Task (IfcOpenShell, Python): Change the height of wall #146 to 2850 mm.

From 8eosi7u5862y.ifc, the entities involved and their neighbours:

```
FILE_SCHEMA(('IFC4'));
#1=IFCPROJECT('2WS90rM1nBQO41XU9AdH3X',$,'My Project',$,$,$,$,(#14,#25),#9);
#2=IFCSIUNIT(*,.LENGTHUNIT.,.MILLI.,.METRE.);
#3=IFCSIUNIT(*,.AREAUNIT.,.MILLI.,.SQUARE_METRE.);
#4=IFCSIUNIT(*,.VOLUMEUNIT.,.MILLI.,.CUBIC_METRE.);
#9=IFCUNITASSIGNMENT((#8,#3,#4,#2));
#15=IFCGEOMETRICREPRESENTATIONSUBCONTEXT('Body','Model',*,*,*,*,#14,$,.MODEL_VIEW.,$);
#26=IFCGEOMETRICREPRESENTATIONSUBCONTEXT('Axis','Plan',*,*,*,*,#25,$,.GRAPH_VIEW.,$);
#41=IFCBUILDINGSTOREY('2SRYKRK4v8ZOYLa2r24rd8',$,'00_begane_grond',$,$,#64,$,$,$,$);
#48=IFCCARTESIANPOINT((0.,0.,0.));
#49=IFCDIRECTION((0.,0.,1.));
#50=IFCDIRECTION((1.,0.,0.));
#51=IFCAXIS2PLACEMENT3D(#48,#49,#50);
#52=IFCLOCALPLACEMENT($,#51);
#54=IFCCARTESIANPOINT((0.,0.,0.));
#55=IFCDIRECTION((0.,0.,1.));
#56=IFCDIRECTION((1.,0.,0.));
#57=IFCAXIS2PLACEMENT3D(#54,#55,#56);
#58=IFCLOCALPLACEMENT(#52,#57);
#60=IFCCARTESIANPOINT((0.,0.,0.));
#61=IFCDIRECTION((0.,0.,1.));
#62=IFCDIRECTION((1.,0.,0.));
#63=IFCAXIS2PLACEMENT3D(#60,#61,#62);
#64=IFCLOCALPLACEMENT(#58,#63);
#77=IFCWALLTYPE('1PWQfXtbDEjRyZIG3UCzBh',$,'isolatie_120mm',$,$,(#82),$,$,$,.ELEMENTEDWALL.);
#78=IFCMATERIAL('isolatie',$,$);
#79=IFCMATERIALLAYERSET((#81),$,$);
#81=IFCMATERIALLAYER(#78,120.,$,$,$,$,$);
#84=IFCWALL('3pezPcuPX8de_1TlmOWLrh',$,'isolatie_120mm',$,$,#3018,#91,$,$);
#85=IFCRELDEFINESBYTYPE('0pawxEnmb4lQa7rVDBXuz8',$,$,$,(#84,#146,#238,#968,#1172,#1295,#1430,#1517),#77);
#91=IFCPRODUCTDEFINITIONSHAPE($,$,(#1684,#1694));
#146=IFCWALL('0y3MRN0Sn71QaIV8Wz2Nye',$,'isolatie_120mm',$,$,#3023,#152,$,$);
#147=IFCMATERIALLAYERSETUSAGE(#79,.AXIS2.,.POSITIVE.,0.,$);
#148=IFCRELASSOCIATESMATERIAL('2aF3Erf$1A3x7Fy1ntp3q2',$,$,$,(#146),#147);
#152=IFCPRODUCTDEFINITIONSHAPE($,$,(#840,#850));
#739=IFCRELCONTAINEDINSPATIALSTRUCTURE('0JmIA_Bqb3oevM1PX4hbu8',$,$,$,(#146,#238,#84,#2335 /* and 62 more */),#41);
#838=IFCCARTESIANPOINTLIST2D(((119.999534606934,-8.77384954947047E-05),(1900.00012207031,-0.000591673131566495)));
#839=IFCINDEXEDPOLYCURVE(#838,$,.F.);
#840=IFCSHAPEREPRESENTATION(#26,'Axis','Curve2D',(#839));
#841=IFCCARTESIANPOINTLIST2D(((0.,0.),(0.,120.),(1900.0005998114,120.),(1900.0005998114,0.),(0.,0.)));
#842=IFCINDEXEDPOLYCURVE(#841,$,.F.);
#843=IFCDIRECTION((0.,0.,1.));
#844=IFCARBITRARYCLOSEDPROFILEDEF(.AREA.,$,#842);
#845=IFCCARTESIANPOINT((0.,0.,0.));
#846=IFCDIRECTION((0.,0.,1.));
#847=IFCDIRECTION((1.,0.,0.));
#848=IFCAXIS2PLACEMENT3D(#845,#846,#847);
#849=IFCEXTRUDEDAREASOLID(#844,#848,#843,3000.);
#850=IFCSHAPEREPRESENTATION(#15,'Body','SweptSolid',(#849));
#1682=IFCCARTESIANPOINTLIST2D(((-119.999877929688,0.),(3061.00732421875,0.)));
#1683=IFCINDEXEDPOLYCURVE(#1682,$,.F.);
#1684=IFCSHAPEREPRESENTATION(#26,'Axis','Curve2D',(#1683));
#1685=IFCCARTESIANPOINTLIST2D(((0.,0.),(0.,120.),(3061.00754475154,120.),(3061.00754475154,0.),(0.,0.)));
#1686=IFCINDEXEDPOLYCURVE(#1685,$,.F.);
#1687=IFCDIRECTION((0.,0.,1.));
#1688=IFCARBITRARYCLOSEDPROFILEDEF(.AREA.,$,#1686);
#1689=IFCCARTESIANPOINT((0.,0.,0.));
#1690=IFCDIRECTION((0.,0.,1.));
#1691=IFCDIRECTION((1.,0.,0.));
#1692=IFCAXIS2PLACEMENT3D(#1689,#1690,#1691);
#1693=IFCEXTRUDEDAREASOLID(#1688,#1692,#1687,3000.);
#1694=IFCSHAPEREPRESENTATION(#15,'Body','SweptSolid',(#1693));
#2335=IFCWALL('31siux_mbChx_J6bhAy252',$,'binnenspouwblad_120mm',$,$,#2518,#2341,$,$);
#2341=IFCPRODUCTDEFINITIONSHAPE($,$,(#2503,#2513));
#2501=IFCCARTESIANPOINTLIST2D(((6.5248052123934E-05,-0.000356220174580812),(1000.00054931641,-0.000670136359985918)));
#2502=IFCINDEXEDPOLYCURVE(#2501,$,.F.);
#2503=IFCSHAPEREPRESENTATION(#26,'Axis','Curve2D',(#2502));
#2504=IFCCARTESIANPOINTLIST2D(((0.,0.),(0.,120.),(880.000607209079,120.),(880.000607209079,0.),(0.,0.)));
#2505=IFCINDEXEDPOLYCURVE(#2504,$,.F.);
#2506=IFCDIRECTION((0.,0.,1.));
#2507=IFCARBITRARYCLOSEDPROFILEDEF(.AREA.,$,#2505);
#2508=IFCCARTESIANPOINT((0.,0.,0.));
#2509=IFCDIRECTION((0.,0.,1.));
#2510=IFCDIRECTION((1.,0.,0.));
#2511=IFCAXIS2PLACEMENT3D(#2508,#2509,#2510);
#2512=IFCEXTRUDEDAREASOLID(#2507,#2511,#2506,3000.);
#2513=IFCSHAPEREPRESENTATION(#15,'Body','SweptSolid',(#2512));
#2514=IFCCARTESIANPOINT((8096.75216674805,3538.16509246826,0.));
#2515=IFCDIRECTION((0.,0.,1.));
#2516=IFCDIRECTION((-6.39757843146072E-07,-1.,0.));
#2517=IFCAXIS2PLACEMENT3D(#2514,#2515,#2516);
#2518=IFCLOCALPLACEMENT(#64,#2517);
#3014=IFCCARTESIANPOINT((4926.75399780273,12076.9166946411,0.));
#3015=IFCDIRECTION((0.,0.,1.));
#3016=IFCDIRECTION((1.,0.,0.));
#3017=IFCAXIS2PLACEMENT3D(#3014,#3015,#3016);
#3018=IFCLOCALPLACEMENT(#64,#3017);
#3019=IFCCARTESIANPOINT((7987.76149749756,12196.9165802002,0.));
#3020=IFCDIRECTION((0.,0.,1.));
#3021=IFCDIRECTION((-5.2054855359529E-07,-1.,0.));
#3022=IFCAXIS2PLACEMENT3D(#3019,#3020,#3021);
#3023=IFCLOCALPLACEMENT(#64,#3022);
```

```python
import ifcopenshell
import ifcopenshell.geom
import ifcopenshell.util.representation
import ifcopenshell.util.shape
import ifcopenshell.util.unit

model = ifcopenshell.open("8eosi7u5862y.ifc")
unit_scale = ifcopenshell.util.unit.calculate_unit_scale(model)
settings = ifcopenshell.geom.settings()


def volume(element):
    """Net volume in cubic metres, openings subtracted."""
    shape = ifcopenshell.geom.create_shape(settings, element)
    return ifcopenshell.util.shape.get_volume(shape.geometry)


wall = model.by_id(146)
before = volume(wall)

body = ifcopenshell.util.representation.get_representation(wall, "Model", "Body")
solid = body.Items[0]
old_height = solid.Depth
solid.Depth = 2.85 / unit_scale
after = volume(wall)

print(f"height {old_height:g} -> {solid.Depth:g}, volume {before:.3f} -> {after:.3f} m3")

model.write("8eosi7u5862y_updated.ifc")
```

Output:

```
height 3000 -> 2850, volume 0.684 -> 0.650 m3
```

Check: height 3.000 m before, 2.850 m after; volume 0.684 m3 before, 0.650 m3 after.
